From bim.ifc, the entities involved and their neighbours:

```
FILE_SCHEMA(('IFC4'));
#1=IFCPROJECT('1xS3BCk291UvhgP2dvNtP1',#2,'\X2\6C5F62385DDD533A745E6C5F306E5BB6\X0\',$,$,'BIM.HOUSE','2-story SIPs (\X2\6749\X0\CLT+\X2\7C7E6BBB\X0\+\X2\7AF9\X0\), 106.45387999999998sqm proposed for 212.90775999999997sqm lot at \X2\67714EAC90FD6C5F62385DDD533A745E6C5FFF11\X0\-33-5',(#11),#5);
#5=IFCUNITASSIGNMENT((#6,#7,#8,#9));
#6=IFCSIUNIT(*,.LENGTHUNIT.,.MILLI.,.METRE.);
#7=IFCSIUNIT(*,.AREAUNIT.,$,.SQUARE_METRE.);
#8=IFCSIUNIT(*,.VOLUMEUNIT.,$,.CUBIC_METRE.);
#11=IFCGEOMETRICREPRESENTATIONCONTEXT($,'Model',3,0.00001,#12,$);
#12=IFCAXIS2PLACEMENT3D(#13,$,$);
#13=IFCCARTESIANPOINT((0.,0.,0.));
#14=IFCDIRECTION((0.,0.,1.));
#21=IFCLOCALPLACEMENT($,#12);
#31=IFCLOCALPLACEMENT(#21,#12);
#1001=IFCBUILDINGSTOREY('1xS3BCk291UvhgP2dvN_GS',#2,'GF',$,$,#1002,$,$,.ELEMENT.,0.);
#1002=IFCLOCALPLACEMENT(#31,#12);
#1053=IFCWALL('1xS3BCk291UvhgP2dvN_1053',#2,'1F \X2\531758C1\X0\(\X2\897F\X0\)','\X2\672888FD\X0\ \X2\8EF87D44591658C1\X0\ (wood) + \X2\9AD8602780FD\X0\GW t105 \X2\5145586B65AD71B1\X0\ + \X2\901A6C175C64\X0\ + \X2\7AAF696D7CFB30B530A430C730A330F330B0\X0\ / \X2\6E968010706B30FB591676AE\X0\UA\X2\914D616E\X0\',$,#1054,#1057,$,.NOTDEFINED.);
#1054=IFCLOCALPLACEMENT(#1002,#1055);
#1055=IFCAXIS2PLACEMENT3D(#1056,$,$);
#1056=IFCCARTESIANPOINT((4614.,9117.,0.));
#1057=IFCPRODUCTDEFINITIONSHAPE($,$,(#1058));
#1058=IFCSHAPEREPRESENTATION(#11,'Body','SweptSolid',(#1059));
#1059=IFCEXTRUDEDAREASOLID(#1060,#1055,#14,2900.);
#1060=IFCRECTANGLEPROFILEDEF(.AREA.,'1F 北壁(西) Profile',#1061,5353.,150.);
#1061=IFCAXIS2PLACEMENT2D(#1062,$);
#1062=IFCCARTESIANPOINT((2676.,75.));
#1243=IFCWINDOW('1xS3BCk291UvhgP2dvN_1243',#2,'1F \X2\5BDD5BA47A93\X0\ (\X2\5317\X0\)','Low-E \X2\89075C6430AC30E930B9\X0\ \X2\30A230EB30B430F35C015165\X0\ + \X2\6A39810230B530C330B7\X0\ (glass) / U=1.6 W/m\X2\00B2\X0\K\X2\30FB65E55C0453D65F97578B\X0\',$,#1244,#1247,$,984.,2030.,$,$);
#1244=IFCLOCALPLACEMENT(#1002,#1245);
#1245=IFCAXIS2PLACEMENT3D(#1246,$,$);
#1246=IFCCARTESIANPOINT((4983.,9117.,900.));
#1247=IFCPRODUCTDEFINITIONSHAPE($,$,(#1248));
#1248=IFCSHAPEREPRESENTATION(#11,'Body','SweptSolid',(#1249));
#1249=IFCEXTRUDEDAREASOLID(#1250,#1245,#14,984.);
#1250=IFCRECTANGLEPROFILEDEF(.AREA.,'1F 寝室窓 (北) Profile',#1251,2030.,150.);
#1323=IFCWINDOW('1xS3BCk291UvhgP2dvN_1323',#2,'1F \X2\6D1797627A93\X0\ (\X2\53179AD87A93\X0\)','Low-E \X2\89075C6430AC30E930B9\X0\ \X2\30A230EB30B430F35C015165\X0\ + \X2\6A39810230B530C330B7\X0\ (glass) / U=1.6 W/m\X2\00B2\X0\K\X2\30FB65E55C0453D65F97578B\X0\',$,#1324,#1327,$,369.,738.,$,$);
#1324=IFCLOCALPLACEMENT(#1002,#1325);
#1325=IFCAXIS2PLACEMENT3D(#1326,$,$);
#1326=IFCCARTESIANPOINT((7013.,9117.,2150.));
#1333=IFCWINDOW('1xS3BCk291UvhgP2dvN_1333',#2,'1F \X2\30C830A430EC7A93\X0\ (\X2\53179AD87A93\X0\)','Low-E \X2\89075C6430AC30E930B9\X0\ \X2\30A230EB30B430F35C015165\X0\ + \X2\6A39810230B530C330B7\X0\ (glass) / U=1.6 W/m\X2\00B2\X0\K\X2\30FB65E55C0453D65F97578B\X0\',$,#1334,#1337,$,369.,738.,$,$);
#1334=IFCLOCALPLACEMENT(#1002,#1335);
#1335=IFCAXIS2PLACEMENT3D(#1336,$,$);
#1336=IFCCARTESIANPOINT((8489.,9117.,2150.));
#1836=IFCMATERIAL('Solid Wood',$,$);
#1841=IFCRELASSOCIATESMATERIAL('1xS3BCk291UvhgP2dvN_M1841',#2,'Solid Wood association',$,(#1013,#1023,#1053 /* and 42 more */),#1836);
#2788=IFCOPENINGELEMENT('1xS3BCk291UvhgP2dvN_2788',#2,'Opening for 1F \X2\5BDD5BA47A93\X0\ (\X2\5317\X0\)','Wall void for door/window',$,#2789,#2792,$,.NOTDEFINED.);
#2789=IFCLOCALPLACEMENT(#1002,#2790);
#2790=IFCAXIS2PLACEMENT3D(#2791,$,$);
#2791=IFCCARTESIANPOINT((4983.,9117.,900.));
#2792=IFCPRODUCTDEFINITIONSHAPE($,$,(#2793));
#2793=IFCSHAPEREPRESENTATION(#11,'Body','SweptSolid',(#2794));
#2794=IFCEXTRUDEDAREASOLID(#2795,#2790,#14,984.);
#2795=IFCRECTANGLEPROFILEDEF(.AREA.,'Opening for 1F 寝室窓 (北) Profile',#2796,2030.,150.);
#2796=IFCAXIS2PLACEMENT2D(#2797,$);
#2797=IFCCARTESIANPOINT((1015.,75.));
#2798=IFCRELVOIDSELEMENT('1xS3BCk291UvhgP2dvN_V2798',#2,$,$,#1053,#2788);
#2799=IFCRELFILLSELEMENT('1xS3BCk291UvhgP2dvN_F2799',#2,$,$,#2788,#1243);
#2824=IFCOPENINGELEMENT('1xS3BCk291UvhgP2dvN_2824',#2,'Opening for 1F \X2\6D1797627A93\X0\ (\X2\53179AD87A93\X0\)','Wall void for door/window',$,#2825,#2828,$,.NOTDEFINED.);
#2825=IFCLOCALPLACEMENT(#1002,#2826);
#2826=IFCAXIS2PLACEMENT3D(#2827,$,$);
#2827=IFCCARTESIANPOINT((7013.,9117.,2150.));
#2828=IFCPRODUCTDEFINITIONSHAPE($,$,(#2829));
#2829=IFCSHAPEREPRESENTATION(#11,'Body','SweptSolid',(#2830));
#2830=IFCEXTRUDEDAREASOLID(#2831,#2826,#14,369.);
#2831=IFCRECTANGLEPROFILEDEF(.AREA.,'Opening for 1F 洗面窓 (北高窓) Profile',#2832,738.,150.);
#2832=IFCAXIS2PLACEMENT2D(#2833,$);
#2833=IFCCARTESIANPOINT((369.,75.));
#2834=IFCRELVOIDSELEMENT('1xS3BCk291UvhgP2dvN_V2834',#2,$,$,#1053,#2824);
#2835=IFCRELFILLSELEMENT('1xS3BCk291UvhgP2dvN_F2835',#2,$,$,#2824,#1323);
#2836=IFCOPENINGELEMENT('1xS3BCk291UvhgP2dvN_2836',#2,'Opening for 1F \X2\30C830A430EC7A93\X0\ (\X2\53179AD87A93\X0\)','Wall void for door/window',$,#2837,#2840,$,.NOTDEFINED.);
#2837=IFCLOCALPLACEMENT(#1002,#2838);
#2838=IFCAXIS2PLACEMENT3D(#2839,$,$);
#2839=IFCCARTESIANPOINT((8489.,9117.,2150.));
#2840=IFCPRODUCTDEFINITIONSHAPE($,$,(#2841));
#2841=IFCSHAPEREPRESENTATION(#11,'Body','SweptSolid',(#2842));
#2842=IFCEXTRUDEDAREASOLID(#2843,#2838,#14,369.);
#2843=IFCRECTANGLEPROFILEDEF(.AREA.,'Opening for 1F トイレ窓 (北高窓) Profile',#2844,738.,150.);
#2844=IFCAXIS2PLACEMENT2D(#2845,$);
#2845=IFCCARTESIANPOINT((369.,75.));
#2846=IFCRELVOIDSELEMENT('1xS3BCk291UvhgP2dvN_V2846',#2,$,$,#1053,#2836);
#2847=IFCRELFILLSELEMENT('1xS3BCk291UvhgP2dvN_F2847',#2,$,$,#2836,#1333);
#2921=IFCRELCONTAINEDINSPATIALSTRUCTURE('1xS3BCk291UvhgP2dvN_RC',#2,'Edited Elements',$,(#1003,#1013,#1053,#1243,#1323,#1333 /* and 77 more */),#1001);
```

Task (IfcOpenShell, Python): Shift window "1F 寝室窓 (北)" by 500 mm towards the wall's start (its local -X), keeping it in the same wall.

```python
import ifcopenshell
import ifcopenshell.api.geometry
import ifcopenshell.util.placement
import ifcopenshell.util.unit

model = ifcopenshell.open("bim.ifc")
unit_scale = ifcopenshell.util.unit.calculate_unit_scale(model)

window = model.by_guid("1xS3BCk291UvhgP2dvN_1243")
opening = window.FillsVoids[0].RelatingOpeningElement
wall = opening.VoidsElements[0].RelatingBuildingElement

wall_matrix = ifcopenshell.util.placement.get_local_placement(wall.ObjectPlacement)
shift = wall_matrix[:3, 0] * -0.5 / unit_scale
before = ifcopenshell.util.placement.get_local_placement(window.ObjectPlacement)[:3, 3].copy()

# The window is not placed relative to its opening, so move both.
for product in (opening, window):
    matrix = ifcopenshell.util.placement.get_local_placement(product.ObjectPlacement)
    matrix[:3, 3] += shift
    ifcopenshell.api.geometry.edit_object_placement(model, product=product, matrix=matrix, is_si=False)

after = ifcopenshell.util.placement.get_local_placement(window.ObjectPlacement)[:3, 3]
print("window moved by", (after - before).round(3) + 0.0)

model.write("bim_v2.ifc")
```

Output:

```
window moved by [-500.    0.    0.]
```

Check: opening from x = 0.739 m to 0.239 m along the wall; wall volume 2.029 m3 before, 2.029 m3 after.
